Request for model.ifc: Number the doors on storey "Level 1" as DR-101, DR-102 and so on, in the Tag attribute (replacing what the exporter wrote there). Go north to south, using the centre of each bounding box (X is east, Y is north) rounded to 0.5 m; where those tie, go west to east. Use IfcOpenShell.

First a look at what the model holds.

```python
import ifcopenshell
import ifcopenshell.util.element
import ifcopenshell.util.placement

model = ifcopenshell.open("model.ifc")
print(model.schema)
storey = next(s for s in model.by_type("IfcBuildingStorey") if s.Name == "Level 1")
doors = [e for e in ifcopenshell.util.element.get_decomposition(storey) if e.is_a("IfcDoor")]
for e in sorted(doors, key=lambda e: e.id()):
    origin = ifcopenshell.util.placement.get_local_placement(e.ObjectPlacement)[:3, 3]
    print(e.id(), e.Tag, e.Name, origin.round(2) + 0.0, sep=" | ")
```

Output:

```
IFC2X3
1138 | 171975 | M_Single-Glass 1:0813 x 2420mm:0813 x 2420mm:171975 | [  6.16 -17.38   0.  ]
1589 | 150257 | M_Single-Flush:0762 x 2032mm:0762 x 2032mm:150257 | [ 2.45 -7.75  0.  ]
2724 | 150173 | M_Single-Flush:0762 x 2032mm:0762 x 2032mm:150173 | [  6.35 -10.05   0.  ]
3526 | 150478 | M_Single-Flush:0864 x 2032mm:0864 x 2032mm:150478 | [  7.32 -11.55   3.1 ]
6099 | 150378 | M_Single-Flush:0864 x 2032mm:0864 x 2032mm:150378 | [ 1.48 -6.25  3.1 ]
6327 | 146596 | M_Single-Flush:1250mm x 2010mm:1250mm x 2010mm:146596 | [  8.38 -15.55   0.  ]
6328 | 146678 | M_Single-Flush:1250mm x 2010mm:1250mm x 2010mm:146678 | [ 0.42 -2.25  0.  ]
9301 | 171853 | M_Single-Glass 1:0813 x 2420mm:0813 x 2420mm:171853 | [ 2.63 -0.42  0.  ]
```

```python
import ifcopenshell
import ifcopenshell.geom
import ifcopenshell.util.element
import ifcopenshell.util.shape

model = ifcopenshell.open("model.ifc")
settings = ifcopenshell.geom.settings()
settings.set("use-world-coords", True)


def centre(element):
    shape = ifcopenshell.geom.create_shape(settings, element)
    return ifcopenshell.util.shape.get_bbox_centroid(shape.geometry)


storey = next(s for s in model.by_type("IfcBuildingStorey") if s.Name == "Level 1")
doors = [e for e in ifcopenshell.util.element.get_decomposition(storey) if e.is_a("IfcDoor")]

# Insertion points can sit at a corner or the storey origin, so sort by the geometry (in metres).
centres = {e: centre(e) for e in doors}
doors.sort(key=lambda e: (-round(centres[e][1] / 0.5), centres[e][0]))

for i, e in enumerate(doors, start=1):
    number = f"DR-1{i:02d}"
    e.Tag = number
    print(e.id(), number)

model.write("model-out.ifc")
```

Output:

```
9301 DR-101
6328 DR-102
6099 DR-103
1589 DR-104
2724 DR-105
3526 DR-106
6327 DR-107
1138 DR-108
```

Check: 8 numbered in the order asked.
